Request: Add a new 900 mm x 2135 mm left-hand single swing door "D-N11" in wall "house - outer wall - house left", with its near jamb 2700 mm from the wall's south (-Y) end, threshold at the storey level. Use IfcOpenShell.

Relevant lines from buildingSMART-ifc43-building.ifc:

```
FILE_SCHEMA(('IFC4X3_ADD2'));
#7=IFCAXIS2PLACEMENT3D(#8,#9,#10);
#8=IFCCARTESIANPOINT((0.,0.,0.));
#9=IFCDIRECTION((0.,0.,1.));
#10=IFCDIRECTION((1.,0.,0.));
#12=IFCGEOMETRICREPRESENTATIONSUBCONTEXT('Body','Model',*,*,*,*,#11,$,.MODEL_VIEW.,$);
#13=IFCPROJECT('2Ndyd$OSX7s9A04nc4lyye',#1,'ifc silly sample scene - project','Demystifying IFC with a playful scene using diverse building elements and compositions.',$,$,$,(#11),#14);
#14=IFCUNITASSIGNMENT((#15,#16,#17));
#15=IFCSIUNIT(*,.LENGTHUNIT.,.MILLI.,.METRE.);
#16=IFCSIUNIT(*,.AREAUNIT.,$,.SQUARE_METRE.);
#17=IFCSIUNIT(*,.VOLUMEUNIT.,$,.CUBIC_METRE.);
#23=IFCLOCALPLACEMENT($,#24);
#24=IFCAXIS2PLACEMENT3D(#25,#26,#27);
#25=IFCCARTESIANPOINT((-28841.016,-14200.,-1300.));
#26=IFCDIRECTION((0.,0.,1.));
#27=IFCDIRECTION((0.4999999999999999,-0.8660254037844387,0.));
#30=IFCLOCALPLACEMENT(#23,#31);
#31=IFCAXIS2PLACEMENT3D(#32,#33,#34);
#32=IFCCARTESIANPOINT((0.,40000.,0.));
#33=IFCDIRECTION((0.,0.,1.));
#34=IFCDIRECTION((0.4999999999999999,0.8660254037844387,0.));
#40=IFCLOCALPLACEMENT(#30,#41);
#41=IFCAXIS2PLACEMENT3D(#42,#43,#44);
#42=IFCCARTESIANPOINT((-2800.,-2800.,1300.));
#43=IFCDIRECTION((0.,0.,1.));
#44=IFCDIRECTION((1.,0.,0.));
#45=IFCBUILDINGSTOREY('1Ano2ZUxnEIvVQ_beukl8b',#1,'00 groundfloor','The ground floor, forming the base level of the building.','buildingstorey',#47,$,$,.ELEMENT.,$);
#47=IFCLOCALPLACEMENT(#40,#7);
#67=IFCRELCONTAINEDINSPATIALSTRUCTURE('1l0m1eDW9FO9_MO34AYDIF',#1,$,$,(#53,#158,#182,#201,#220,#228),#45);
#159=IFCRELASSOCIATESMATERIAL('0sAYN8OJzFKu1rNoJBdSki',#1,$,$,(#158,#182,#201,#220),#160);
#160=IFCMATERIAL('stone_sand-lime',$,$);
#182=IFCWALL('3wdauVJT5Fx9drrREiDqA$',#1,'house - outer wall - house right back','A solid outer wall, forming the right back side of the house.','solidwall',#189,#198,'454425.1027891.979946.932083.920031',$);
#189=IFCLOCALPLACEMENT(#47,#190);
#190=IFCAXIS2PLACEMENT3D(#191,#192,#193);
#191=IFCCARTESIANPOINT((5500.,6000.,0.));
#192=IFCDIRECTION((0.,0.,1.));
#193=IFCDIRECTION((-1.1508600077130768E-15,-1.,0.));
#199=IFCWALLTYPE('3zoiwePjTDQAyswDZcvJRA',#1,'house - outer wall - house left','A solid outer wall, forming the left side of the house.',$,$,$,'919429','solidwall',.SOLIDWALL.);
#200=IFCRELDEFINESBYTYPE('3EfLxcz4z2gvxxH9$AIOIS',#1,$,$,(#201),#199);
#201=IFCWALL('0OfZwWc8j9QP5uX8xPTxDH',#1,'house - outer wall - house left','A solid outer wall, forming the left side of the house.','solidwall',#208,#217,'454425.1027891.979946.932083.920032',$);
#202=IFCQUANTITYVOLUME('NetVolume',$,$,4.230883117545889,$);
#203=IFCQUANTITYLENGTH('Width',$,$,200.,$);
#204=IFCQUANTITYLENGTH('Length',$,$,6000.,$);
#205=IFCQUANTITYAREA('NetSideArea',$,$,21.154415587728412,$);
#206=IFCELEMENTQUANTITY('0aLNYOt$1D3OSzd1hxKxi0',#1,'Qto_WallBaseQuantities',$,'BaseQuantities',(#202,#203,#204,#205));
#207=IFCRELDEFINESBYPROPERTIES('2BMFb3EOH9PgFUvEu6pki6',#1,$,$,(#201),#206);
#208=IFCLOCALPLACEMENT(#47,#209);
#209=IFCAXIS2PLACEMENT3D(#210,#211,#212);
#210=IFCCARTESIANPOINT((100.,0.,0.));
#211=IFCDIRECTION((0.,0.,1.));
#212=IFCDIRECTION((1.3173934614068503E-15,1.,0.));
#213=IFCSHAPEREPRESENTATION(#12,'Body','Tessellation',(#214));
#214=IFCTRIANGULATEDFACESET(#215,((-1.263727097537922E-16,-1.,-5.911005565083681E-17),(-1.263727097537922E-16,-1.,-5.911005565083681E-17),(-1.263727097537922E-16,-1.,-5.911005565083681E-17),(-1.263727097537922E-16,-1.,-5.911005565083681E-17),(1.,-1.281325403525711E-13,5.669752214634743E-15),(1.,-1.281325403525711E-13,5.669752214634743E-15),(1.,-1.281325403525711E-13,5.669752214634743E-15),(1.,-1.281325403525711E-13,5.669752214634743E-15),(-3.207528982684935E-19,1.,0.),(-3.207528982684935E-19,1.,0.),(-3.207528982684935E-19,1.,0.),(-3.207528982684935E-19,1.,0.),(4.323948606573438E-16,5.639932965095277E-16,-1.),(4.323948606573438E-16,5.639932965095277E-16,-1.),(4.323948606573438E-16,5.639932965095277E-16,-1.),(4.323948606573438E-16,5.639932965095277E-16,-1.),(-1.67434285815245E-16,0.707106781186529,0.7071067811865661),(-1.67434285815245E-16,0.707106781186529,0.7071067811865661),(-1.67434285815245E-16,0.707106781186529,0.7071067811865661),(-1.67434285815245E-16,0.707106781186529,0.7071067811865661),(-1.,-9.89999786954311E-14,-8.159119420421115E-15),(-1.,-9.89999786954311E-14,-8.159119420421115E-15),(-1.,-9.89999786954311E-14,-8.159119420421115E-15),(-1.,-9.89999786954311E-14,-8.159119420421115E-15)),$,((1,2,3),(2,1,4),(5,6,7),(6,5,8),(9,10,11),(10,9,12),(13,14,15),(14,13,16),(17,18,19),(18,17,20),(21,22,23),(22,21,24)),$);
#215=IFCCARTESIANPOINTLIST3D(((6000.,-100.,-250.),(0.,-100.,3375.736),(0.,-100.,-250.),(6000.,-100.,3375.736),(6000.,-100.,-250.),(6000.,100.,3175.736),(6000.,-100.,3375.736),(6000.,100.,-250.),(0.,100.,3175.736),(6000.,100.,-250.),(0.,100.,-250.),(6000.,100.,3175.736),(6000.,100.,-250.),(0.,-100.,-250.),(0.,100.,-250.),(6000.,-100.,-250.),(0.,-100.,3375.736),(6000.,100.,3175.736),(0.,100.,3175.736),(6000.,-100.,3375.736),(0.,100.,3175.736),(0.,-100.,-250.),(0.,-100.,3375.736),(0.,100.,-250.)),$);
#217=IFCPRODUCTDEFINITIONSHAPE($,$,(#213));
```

```python
import numpy as np
import ifcopenshell
import ifcopenshell.api.feature
import ifcopenshell.api.geometry
import ifcopenshell.api.pset
import ifcopenshell.api.root
import ifcopenshell.api.spatial
import ifcopenshell.geom
import ifcopenshell.util.element
import ifcopenshell.util.placement
import ifcopenshell.util.representation
import ifcopenshell.util.shape
import ifcopenshell.util.unit

model = ifcopenshell.open("buildingSMART-ifc43-building.ifc")
unit_scale = ifcopenshell.util.unit.calculate_unit_scale(model)
area_scale = ifcopenshell.util.unit.calculate_unit_scale(model, "AREAUNIT")
volume_scale = ifcopenshell.util.unit.calculate_unit_scale(model, "VOLUMEUNIT")
settings = ifcopenshell.geom.settings()


def volume(element):
    """Net volume in cubic metres, openings subtracted."""
    shape = ifcopenshell.geom.create_shape(settings, element)
    return ifcopenshell.util.shape.get_volume(shape.geometry)


wall = model.by_guid("0OfZwWc8j9QP5uX8xPTxDH")
storey = ifcopenshell.util.element.get_container(wall, ifc_class="IfcBuildingStorey")
context = ifcopenshell.util.representation.get_context(model, "Model", "Body", "MODEL_VIEW")
before = volume(wall)

width, height, from_end, sill = 0.9, 2.135, 2.7, 0.0  # metres

# The wall runs along its own X axis, and the end named is its -X end.
wall_shape = ifcopenshell.geom.create_shape(settings, wall)
x, y, z = ifcopenshell.util.shape.get_vertices(wall_shape.geometry).T
start = x.min() + from_end
face, thickness = float(y.min()), float(y.max() - y.min())
wall_matrix = ifcopenshell.util.placement.get_local_placement(wall.ObjectPlacement)
level = ifcopenshell.util.placement.get_local_placement(storey.ObjectPlacement)[2, 3]


def in_wall(x, y):
    """Placement at x, y metres in the wall's axes, at sill height."""
    matrix = wall_matrix.copy()
    matrix[:, 3] = wall_matrix @ np.array([x / unit_scale, y / unit_scale, 0.0, 1.0])
    matrix[2, 3] = level + sill / unit_scale
    return matrix


# Opening: a box that overshoots both wall faces by 50 mm.
opening = ifcopenshell.api.root.create_entity(model, ifc_class="IfcOpeningElement", predefined_type="OPENING")
box = ifcopenshell.api.geometry.add_wall_representation(
    model, context=context, length=width, height=height, thickness=thickness + 0.1
)
ifcopenshell.api.geometry.assign_representation(model, product=opening, representation=box)
ifcopenshell.api.geometry.edit_object_placement(model, product=opening, matrix=in_wall(start, face - 0.05), is_si=False)
ifcopenshell.api.feature.add_feature(model, feature=opening, element=wall)

door = ifcopenshell.api.root.create_entity(model, ifc_class="IfcDoor", name="D-N11", predefined_type="DOOR")
door.OverallWidth, door.OverallHeight = width / unit_scale, height / unit_scale
door.OperationType = "SINGLE_SWING_LEFT"
body = ifcopenshell.api.geometry.add_door_representation(
    model,
    context=context,
    overall_width=door.OverallWidth,
    overall_height=door.OverallHeight,
    operation_type="SINGLE_SWING_LEFT",
    lining_properties={"LiningDepth": thickness / unit_scale, "ThresholdDepth": thickness / unit_scale},
)
ifcopenshell.api.geometry.assign_representation(model, product=door, representation=body)
ifcopenshell.api.spatial.assign_container(model, products=[door], relating_structure=storey)
ifcopenshell.api.feature.add_filling(model, opening=opening, element=door)

# The lining spans the wall, so the door starts at the wall face.
ifcopenshell.api.geometry.edit_object_placement(model, product=door, matrix=in_wall(start, face), is_si=False)

after = volume(wall)

# Update the wall's stored quantities.
qto = model.by_id(ifcopenshell.util.element.get_pset(wall, "Qto_WallBaseQuantities", should_inherit=False)["id"])
ifcopenshell.api.pset.edit_qto(model, qto=qto, properties={
    "NetVolume": after / volume_scale,
    "NetSideArea": after / thickness / area_scale,
})

print(f"wall volume {before:.3f} -> {after:.3f} m3")

model.write("buildingSMART-ifc43-building_rev.ifc")
```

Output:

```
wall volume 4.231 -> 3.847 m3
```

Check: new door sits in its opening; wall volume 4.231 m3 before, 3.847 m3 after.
